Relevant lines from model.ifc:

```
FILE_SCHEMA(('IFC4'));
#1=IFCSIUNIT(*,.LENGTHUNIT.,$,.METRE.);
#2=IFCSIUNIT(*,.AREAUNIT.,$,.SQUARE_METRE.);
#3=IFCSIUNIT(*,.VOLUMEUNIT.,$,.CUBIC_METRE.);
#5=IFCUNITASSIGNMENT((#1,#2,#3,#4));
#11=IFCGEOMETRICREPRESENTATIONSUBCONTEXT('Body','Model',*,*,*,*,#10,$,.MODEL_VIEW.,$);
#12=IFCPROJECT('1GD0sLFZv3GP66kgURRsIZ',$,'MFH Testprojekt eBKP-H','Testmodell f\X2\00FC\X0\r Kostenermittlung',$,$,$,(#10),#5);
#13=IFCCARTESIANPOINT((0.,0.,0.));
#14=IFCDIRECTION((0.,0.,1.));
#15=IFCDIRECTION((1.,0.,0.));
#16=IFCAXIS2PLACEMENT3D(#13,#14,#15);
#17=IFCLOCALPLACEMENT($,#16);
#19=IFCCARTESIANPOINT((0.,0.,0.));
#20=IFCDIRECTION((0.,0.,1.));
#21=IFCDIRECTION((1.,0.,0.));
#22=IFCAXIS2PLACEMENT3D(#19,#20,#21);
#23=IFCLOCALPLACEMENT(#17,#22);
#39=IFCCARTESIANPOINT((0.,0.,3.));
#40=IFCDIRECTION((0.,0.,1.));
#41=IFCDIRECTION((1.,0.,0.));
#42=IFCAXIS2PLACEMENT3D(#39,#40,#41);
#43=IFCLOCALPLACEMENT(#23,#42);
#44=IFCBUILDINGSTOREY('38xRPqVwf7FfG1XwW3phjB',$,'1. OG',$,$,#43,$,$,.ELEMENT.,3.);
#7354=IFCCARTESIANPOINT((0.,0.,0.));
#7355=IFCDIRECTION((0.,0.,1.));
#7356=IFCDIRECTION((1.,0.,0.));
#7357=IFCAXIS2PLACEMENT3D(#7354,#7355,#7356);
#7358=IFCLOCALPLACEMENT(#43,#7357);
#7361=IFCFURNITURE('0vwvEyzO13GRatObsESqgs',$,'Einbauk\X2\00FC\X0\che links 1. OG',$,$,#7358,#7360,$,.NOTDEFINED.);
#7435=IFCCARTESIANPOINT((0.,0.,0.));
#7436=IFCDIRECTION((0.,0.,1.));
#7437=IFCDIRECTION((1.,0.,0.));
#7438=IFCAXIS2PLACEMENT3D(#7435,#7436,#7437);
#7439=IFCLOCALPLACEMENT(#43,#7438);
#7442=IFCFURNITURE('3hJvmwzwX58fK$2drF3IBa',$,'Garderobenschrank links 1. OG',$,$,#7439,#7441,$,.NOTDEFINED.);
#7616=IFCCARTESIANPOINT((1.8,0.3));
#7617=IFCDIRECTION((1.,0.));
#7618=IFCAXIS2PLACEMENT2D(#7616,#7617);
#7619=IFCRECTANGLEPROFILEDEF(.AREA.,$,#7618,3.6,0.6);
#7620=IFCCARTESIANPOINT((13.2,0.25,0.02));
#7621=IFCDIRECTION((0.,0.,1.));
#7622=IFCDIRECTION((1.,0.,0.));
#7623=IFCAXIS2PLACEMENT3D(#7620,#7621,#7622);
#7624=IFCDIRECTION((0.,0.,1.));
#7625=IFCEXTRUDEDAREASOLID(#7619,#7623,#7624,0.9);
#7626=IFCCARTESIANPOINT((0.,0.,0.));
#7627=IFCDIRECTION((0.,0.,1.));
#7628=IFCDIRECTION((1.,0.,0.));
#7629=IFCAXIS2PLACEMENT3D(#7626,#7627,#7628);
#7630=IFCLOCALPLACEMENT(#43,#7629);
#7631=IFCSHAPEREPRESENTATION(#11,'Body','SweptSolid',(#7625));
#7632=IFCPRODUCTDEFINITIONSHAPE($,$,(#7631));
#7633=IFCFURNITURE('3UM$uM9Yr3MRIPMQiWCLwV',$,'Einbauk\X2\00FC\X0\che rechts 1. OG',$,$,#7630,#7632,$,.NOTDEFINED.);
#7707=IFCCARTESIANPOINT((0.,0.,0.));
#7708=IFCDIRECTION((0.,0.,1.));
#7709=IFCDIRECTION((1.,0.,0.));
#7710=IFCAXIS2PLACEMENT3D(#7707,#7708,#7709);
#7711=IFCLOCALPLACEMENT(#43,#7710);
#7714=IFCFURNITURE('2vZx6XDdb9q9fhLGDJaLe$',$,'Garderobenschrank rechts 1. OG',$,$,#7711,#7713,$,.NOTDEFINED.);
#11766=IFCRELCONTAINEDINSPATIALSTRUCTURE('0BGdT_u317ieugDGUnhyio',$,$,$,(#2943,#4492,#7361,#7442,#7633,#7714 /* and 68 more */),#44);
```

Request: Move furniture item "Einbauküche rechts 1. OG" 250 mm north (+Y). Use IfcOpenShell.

```python
import ifcopenshell
import ifcopenshell.api.geometry
import ifcopenshell.util.placement
import ifcopenshell.util.unit

model = ifcopenshell.open("model.ifc")
unit_scale = ifcopenshell.util.unit.calculate_unit_scale(model)

item = model.by_guid("3UM$uM9Yr3MRIPMQiWCLwV")
matrix = ifcopenshell.util.placement.get_local_placement(item.ObjectPlacement)
matrix[1, 3] += 0.25 / unit_scale
ifcopenshell.api.geometry.edit_object_placement(model, product=item, matrix=matrix, is_si=False)

print(ifcopenshell.util.placement.get_local_placement(item.ObjectPlacement).round(3) + 0.0)

model.write("model_rev.ifc")
```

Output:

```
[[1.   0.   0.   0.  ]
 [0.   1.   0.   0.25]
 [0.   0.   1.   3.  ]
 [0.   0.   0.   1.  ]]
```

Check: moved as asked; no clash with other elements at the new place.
